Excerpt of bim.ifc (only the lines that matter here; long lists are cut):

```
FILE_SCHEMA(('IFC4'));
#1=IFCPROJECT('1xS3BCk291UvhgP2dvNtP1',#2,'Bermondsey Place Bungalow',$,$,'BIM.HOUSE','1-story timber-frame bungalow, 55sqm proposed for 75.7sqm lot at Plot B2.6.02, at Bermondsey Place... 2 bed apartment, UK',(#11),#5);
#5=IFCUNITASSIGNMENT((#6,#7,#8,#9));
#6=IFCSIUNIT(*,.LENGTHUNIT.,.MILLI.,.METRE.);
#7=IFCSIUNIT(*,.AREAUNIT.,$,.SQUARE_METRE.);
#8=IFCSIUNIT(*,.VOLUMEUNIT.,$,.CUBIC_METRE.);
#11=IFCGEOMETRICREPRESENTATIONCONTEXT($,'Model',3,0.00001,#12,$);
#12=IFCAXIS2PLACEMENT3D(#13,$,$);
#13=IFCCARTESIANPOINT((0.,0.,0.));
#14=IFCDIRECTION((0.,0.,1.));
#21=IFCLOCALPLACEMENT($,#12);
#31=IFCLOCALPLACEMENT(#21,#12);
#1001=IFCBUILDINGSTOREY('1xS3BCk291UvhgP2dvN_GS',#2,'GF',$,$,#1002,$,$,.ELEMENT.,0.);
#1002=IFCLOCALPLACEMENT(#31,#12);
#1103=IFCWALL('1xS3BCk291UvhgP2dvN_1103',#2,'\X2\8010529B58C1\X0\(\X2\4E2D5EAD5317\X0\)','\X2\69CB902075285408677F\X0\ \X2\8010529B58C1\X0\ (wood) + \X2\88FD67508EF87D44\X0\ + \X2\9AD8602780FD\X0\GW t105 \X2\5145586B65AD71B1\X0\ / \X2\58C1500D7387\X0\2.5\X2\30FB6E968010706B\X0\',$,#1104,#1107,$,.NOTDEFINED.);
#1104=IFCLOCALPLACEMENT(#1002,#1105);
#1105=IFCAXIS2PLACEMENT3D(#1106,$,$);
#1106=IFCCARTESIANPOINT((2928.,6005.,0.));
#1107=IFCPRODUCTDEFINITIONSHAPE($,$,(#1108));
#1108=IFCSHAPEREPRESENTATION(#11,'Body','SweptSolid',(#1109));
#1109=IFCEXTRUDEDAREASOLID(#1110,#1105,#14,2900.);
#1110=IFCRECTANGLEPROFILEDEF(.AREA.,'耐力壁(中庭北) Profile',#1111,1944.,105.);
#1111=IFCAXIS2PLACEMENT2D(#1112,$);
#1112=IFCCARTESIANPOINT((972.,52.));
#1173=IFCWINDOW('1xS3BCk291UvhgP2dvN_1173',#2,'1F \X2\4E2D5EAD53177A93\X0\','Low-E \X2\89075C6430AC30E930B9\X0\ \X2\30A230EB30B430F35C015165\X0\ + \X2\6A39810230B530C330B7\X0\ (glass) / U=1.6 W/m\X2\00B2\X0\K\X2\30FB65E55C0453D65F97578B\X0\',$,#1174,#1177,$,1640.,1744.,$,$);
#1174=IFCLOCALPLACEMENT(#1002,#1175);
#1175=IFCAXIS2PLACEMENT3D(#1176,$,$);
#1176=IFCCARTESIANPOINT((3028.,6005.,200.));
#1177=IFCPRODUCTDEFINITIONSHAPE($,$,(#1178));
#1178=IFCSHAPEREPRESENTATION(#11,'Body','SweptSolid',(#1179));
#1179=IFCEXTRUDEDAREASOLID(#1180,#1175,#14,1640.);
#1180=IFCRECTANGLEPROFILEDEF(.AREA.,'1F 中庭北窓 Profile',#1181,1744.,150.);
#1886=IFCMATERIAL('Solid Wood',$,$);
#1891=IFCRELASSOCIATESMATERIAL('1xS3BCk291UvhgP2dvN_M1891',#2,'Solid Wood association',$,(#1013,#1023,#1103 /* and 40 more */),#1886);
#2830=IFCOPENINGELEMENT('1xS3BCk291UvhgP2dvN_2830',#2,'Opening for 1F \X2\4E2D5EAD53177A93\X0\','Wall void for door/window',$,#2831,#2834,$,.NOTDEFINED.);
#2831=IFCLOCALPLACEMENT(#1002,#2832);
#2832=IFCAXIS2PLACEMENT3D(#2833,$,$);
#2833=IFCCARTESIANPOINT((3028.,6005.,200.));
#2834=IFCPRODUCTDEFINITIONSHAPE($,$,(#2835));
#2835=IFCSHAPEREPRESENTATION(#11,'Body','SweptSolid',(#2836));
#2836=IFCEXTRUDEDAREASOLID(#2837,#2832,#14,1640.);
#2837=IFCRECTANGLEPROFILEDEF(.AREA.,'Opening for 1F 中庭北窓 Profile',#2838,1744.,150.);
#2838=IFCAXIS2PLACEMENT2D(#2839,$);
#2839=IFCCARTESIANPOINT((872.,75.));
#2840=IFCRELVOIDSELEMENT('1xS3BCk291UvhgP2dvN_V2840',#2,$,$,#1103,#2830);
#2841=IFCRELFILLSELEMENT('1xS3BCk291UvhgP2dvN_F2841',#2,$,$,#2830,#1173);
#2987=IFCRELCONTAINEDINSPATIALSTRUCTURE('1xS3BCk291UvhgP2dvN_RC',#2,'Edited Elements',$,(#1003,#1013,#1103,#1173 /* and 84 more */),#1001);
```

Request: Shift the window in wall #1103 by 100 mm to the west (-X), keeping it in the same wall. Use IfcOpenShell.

```python
import ifcopenshell
import ifcopenshell.api.geometry
import ifcopenshell.util.placement

model = ifcopenshell.open("bim.ifc")

window = model.by_guid("1xS3BCk291UvhgP2dvN_1173")
opening = window.FillsVoids[0].RelatingOpeningElement
wall = opening.VoidsElements[0].RelatingBuildingElement

wall_matrix = ifcopenshell.util.placement.get_local_placement(wall.ObjectPlacement)
shift = wall_matrix[:3, 0] * -100.0
before = ifcopenshell.util.placement.get_local_placement(window.ObjectPlacement)[:3, 3].copy()

# The window is not placed relative to its opening, so move both.
for product in (opening, window):
    matrix = ifcopenshell.util.placement.get_local_placement(product.ObjectPlacement)
    matrix[:3, 3] += shift
    ifcopenshell.api.geometry.edit_object_placement(model, product=product, matrix=matrix, is_si=False)

after = ifcopenshell.util.placement.get_local_placement(window.ObjectPlacement)[:3, 3]
print("window moved by", (after - before).round(3) + 0.0)

model.write("bim_updated.ifc")
```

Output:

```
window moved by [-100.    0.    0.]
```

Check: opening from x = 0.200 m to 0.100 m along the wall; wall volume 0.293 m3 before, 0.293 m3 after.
